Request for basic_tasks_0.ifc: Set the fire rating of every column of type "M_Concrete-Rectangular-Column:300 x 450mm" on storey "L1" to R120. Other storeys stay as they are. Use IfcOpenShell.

First a look at what the model holds.

```python
import ifcopenshell
import ifcopenshell.util.element

model = ifcopenshell.open("basic_tasks_0.ifc")
print(model.schema)
storey = next(s for s in model.by_type("IfcBuildingStorey") if s.Name == "L1")
columns = [e for e in ifcopenshell.util.element.get_decomposition(storey) if e.is_a("IfcColumn")]
seen = {}
for e in columns:
    element_type = ifcopenshell.util.element.get_type(e)
    key = (element_type.Name if element_type != e and element_type else None, ifcopenshell.util.element.get_pset(e, "Pset_ColumnCommon", "FireRating"))
    seen[key] = seen.get(key, 0) + 1
for (name, value), count in sorted(seen.items(), key=str):
    print(count, "x", name, "|", value)
```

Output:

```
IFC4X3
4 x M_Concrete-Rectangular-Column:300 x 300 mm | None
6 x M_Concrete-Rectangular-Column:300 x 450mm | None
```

```python
import ifcopenshell
import ifcopenshell.api.pset
import ifcopenshell.util.element

model = ifcopenshell.open("basic_tasks_0.ifc")

storey = next(s for s in model.by_type("IfcBuildingStorey") if s.Name == "L1")
columns = [e for e in ifcopenshell.util.element.get_decomposition(storey) if e.is_a("IfcColumn")]

count = 0
for e in columns:
    element_type = ifcopenshell.util.element.get_type(e)
    if element_type in (None, e) or element_type.Name != "M_Concrete-Rectangular-Column:300 x 450mm":
        continue
    # add_pset returns the element's existing set when there is one.
    pset = ifcopenshell.api.pset.add_pset(model, product=e, name="Pset_ColumnCommon")
    ifcopenshell.api.pset.edit_pset(model, pset=pset, properties={"FireRating": "R120"})
    count += 1

print(count, "columns updated")

model.write("basic_tasks_0_v2.ifc")
```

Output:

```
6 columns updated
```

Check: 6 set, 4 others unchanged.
